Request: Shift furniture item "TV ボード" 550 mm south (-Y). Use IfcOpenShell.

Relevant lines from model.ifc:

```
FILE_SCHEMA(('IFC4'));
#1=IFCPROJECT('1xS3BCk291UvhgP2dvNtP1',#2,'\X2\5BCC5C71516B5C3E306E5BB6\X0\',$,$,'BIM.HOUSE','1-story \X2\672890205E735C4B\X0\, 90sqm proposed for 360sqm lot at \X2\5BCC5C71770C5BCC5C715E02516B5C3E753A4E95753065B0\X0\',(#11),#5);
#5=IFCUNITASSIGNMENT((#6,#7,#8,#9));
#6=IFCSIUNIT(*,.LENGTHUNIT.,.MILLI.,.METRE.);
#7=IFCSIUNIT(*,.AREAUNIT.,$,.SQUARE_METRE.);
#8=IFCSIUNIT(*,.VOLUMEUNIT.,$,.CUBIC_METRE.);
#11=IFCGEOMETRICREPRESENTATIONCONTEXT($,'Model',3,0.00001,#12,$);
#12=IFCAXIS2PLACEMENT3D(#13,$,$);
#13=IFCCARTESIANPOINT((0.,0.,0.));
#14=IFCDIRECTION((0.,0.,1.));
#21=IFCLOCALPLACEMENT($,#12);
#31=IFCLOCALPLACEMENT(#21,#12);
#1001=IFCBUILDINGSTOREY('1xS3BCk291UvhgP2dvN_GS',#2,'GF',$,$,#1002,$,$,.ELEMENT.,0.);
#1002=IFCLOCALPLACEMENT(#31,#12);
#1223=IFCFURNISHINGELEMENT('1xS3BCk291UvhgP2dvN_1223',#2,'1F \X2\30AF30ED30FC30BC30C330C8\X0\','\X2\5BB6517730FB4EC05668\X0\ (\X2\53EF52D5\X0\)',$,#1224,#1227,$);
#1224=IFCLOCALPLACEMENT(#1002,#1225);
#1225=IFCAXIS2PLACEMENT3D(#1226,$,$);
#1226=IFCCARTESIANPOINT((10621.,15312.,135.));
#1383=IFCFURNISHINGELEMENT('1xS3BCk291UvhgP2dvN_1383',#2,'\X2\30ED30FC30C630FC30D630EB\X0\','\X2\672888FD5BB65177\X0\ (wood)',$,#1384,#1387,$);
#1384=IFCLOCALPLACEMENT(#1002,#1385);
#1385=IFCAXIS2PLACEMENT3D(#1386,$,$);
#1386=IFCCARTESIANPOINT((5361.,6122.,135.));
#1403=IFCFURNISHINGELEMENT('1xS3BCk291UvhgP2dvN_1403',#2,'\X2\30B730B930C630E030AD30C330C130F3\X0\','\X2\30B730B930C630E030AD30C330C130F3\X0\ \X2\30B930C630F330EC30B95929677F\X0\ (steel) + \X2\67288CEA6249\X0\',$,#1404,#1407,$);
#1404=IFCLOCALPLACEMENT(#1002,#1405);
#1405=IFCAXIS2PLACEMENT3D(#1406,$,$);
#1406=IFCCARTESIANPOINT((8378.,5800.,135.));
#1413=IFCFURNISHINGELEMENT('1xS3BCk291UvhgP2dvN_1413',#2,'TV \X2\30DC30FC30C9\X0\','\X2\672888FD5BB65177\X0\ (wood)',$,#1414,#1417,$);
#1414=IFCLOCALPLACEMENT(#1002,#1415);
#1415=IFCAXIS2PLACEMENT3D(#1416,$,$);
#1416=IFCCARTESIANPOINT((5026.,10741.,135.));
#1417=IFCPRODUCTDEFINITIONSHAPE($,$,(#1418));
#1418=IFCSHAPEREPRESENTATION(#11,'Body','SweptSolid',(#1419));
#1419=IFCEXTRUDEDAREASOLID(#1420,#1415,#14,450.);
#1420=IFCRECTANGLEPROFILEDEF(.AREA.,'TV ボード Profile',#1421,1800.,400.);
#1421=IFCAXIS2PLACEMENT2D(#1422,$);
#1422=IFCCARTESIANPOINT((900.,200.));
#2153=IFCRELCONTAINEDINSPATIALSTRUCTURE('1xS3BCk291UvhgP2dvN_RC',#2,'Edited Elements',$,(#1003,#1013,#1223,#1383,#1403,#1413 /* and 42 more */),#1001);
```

```python
import ifcopenshell
import ifcopenshell.api.geometry
import ifcopenshell.util.placement

model = ifcopenshell.open("model.ifc")

item = model.by_id(1413)
matrix = ifcopenshell.util.placement.get_local_placement(item.ObjectPlacement)
matrix[1, 3] -= 550.0
ifcopenshell.api.geometry.edit_object_placement(model, product=item, matrix=matrix, is_si=False)

print(ifcopenshell.util.placement.get_local_placement(item.ObjectPlacement).round(3) + 0.0)

model.write("model_rev.ifc")
```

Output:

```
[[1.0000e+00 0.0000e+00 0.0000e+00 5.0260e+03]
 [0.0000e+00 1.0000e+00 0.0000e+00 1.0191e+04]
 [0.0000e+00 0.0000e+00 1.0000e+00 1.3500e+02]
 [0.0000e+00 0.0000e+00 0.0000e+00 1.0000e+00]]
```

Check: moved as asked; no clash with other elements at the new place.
